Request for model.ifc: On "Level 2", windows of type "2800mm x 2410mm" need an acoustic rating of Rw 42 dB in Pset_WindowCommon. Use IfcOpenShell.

First a look at what the model holds.

```python
import ifcopenshell
import ifcopenshell.util.element

model = ifcopenshell.open("model.ifc")
print(model.schema)
storey = next(s for s in model.by_type("IfcBuildingStorey") if s.Name == "Level 2")
windows = [e for e in ifcopenshell.util.element.get_decomposition(storey) if e.is_a("IfcWindow")]
seen = {}
for e in windows:
    element_type = ifcopenshell.util.element.get_type(e)
    key = (element_type.Name if element_type != e and element_type else None, ifcopenshell.util.element.get_pset(e, "Pset_WindowCommon", "AcousticRating"))
    seen[key] = seen.get(key, 0) + 1
for (name, value), count in sorted(seen.items(), key=str):
    print(count, "x", name, "|", value)
```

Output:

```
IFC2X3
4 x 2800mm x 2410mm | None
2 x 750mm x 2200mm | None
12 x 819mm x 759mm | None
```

```python
import ifcopenshell
import ifcopenshell.api.pset
import ifcopenshell.util.element

model = ifcopenshell.open("model.ifc")

storey = next(s for s in model.by_type("IfcBuildingStorey") if s.Name == "Level 2")
windows = [e for e in ifcopenshell.util.element.get_decomposition(storey) if e.is_a("IfcWindow")]

count = 0
for e in windows:
    element_type = ifcopenshell.util.element.get_type(e)
    if element_type in (None, e) or element_type.Name != "2800mm x 2410mm":
        continue
    # add_pset returns the element's existing set when there is one.
    pset = ifcopenshell.api.pset.add_pset(model, product=e, name="Pset_WindowCommon")
    ifcopenshell.api.pset.edit_pset(model, pset=pset, properties={"AcousticRating": "Rw 42 dB"})
    count += 1

print(count, "windows updated")

model.write("model_rev.ifc")
```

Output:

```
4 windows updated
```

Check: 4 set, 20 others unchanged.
